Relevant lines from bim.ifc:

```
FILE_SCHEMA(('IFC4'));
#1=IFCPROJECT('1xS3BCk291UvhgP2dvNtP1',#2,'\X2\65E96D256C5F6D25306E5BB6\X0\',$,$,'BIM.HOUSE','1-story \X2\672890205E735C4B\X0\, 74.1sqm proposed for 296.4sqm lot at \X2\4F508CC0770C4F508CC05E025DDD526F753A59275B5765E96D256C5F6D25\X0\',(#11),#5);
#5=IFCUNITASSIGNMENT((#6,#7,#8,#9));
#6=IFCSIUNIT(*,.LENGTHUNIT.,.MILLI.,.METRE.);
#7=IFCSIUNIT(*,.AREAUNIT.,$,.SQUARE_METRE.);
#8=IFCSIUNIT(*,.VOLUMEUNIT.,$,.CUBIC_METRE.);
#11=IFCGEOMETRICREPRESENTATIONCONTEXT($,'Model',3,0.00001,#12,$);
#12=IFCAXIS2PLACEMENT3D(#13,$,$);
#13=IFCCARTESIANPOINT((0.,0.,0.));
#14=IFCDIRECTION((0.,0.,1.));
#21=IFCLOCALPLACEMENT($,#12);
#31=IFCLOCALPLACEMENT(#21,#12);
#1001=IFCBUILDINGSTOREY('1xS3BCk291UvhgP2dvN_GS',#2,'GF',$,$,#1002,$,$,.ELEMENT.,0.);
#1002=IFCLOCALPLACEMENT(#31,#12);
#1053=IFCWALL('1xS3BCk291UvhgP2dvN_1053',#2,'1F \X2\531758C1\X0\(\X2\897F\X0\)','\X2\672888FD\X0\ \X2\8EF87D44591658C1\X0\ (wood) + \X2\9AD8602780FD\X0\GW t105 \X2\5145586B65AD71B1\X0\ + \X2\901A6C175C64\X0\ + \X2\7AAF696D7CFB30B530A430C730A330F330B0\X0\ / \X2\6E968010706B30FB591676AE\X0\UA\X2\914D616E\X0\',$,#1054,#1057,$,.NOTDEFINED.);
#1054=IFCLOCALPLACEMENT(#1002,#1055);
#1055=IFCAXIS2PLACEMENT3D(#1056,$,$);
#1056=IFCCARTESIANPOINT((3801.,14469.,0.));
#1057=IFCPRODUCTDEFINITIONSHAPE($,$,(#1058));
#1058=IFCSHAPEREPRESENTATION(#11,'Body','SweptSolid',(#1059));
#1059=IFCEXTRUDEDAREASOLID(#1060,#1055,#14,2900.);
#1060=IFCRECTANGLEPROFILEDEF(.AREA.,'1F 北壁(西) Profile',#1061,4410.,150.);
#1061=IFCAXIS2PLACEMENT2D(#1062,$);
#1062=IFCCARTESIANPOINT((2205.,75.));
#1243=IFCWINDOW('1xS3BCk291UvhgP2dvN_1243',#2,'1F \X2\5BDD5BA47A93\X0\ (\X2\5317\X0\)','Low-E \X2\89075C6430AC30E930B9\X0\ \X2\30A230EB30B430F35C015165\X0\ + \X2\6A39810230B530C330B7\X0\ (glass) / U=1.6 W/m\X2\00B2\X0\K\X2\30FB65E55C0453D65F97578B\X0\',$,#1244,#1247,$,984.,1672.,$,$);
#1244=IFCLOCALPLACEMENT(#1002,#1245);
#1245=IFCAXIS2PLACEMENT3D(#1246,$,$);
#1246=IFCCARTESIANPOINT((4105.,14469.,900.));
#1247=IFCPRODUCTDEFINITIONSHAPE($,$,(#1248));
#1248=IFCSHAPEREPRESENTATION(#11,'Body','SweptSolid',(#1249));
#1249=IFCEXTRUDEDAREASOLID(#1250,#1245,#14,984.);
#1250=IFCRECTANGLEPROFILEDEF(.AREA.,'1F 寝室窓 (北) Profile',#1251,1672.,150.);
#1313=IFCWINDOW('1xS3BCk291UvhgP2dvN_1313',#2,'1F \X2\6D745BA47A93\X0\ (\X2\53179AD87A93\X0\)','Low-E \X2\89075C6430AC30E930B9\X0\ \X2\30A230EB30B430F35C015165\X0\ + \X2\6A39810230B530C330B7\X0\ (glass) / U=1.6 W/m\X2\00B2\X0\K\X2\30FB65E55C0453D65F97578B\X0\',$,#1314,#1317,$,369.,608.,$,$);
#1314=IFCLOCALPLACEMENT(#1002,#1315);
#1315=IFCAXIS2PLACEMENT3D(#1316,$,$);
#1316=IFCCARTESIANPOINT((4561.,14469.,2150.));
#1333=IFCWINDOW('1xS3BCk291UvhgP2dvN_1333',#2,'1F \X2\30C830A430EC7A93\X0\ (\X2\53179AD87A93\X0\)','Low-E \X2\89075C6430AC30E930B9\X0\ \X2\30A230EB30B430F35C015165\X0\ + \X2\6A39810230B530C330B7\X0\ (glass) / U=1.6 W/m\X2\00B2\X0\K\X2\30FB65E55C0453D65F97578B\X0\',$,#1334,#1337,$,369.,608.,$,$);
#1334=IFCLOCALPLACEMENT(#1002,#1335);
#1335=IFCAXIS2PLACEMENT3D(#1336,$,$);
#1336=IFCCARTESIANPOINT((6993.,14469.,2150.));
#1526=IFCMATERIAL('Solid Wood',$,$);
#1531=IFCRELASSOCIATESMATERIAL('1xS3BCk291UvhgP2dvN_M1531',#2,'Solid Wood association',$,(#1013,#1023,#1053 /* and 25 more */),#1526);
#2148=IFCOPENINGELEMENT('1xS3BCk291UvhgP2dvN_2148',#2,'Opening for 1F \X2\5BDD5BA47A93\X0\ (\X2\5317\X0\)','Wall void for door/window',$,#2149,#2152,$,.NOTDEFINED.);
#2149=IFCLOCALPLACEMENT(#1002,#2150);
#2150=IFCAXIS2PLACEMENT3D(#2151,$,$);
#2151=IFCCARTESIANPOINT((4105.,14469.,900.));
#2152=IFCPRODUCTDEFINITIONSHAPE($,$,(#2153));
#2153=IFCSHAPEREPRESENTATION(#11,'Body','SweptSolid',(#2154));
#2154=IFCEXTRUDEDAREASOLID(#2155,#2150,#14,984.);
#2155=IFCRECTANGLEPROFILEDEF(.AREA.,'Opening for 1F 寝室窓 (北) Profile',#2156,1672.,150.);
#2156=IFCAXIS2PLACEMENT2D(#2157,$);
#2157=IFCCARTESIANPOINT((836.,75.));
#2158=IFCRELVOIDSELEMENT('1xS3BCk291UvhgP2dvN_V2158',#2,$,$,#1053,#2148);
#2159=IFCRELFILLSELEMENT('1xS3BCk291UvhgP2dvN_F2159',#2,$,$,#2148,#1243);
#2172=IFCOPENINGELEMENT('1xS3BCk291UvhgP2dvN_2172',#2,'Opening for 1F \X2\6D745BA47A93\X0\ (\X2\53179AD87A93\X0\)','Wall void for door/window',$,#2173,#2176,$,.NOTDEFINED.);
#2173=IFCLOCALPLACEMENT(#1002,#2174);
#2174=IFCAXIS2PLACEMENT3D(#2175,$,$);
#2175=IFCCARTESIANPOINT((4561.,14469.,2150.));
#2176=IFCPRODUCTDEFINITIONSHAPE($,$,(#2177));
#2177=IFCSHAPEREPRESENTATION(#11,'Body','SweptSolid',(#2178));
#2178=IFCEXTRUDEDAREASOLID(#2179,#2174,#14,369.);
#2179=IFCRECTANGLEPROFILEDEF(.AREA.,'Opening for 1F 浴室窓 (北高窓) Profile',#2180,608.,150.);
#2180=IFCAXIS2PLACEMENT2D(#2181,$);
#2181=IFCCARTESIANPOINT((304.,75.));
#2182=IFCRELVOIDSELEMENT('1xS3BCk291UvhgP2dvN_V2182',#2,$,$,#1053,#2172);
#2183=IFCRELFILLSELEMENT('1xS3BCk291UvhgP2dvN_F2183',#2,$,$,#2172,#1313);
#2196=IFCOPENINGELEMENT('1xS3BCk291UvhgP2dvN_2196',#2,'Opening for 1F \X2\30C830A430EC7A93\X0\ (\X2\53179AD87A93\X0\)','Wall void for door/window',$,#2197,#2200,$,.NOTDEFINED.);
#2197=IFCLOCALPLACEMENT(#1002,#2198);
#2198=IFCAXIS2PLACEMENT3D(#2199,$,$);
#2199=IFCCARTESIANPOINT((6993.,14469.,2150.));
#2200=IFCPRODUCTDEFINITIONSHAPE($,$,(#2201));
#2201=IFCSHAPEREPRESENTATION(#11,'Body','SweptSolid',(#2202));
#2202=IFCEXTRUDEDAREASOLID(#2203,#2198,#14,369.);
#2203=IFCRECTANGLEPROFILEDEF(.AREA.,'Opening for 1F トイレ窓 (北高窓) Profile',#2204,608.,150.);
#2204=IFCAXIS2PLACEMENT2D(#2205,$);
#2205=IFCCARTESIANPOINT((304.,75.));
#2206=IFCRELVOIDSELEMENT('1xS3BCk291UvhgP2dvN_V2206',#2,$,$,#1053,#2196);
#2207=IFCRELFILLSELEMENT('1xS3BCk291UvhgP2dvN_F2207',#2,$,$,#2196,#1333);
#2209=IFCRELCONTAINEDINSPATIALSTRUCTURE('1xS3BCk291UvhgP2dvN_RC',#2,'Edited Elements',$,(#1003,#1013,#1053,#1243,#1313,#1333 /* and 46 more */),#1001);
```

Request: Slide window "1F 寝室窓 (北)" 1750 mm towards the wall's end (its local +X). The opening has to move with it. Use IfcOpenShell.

```python
import ifcopenshell
import ifcopenshell.api.geometry
import ifcopenshell.util.placement
import ifcopenshell.util.unit

model = ifcopenshell.open("bim.ifc")
unit_scale = ifcopenshell.util.unit.calculate_unit_scale(model)

window = model.by_guid("1xS3BCk291UvhgP2dvN_1243")
opening = window.FillsVoids[0].RelatingOpeningElement
wall = opening.VoidsElements[0].RelatingBuildingElement

wall_matrix = ifcopenshell.util.placement.get_local_placement(wall.ObjectPlacement)
shift = wall_matrix[:3, 0] * 1.75 / unit_scale
before = ifcopenshell.util.placement.get_local_placement(window.ObjectPlacement)[:3, 3].copy()

# The window is not placed relative to its opening, so move both.
for product in (opening, window):
    matrix = ifcopenshell.util.placement.get_local_placement(product.ObjectPlacement)
    matrix[:3, 3] += shift
    ifcopenshell.api.geometry.edit_object_placement(model, product=product, matrix=matrix, is_si=False)

after = ifcopenshell.util.placement.get_local_placement(window.ObjectPlacement)[:3, 3]
print("window moved by", (after - before).round(3) + 0.0)

model.write("bim-out.ifc")
```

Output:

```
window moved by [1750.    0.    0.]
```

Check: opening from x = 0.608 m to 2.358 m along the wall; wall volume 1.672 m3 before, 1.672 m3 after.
